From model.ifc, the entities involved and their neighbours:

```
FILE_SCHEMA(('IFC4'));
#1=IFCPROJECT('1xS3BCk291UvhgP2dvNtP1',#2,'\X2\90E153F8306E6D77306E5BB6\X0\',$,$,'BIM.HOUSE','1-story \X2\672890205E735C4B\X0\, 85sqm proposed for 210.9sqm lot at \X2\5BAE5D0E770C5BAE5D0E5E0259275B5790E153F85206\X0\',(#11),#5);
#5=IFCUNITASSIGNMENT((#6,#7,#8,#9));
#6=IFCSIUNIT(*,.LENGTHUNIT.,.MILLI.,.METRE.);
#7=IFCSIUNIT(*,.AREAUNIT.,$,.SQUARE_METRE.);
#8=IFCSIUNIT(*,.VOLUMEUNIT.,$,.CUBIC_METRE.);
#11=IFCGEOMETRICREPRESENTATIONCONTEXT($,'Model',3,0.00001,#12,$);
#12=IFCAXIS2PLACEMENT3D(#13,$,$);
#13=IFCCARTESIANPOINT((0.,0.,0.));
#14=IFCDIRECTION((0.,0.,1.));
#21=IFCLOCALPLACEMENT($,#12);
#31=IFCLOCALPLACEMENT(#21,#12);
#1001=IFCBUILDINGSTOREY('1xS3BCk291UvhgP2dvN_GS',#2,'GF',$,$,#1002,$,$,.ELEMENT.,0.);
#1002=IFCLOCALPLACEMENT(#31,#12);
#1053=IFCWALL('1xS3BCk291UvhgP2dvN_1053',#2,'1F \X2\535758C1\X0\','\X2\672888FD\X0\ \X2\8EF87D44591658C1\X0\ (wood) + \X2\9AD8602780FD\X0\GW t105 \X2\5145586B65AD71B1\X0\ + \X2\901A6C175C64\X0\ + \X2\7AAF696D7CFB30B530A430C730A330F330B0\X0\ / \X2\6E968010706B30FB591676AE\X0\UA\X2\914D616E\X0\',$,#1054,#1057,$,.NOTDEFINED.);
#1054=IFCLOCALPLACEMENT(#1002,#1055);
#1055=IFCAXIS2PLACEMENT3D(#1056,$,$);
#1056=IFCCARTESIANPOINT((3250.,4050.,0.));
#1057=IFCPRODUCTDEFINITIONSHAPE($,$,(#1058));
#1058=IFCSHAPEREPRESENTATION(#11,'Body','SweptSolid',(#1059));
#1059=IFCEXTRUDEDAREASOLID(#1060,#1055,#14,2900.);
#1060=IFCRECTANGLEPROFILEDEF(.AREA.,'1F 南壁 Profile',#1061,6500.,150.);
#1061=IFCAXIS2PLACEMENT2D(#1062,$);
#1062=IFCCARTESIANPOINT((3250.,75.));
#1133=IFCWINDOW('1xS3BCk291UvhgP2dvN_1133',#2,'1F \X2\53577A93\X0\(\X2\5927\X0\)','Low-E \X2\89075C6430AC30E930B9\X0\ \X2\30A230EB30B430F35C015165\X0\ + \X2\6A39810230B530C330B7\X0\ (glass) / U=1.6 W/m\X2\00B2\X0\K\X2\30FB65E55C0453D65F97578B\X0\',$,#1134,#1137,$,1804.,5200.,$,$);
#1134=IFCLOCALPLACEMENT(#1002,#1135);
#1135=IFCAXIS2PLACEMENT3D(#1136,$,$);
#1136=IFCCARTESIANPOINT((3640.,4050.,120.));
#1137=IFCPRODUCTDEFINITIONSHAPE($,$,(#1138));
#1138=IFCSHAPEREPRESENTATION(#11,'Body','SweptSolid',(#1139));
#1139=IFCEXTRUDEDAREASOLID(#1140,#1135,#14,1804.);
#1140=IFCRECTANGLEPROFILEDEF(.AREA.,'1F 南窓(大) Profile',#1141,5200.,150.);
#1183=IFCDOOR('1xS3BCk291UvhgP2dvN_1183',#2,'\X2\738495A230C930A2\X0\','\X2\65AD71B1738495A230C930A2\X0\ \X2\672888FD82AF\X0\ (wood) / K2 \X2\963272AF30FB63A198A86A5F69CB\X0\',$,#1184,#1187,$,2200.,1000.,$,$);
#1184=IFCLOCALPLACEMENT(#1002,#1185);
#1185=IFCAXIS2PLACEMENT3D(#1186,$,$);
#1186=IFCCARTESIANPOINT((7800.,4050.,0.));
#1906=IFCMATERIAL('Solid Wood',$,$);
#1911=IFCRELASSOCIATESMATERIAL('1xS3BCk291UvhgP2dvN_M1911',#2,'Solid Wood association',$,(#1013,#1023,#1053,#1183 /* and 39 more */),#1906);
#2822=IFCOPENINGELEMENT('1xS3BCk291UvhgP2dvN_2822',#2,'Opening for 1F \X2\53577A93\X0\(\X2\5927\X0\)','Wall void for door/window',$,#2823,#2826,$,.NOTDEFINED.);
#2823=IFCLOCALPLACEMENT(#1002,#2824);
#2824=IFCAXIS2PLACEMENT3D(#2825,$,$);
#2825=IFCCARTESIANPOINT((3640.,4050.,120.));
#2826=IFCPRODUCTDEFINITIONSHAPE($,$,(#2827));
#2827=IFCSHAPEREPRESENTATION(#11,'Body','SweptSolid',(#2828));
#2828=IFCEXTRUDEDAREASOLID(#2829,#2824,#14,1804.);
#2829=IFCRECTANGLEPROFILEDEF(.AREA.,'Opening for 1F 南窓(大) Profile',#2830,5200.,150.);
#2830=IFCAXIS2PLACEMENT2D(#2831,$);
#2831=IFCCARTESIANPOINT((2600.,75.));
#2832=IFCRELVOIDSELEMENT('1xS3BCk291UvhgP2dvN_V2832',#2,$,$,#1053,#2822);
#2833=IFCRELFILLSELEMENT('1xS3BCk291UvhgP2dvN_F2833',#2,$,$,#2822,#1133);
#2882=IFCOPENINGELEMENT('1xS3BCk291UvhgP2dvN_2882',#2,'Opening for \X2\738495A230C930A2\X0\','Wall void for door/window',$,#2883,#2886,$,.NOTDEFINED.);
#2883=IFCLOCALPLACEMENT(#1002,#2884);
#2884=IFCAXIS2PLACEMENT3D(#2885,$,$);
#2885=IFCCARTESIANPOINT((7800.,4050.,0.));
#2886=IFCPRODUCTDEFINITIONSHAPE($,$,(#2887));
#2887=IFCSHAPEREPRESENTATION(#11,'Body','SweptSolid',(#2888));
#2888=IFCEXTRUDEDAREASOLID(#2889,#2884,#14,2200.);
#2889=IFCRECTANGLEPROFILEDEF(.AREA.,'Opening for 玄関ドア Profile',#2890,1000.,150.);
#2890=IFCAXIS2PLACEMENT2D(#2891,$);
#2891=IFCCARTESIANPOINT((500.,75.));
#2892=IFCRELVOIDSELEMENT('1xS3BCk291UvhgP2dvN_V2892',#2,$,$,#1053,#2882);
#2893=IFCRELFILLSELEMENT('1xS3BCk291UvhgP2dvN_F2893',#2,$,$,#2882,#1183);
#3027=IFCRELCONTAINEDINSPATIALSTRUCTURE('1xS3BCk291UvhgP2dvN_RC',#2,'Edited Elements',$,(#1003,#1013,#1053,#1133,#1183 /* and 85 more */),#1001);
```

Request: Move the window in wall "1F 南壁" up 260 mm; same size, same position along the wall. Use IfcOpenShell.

```python
import numpy as np
import ifcopenshell
import ifcopenshell.api.geometry
import ifcopenshell.util.placement
import ifcopenshell.util.unit

model = ifcopenshell.open("model.ifc")
unit_scale = ifcopenshell.util.unit.calculate_unit_scale(model)

window = model.by_id(1133)
opening = window.FillsVoids[0].RelatingOpeningElement
dz = 260.0

shift = np.array([0.0, 0.0, dz])
# The window is not placed relative to its opening, so move both.
for product in (opening, window):
    matrix = ifcopenshell.util.placement.get_local_placement(product.ObjectPlacement)
    matrix[:3, 3] += shift
    ifcopenshell.api.geometry.edit_object_placement(model, product=product, matrix=matrix, is_si=False)

print(f"moved by {dz * unit_scale:+.3f} m")

model.write("model_rev.ifc")
```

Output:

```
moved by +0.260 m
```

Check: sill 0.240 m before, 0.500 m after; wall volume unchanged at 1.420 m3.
